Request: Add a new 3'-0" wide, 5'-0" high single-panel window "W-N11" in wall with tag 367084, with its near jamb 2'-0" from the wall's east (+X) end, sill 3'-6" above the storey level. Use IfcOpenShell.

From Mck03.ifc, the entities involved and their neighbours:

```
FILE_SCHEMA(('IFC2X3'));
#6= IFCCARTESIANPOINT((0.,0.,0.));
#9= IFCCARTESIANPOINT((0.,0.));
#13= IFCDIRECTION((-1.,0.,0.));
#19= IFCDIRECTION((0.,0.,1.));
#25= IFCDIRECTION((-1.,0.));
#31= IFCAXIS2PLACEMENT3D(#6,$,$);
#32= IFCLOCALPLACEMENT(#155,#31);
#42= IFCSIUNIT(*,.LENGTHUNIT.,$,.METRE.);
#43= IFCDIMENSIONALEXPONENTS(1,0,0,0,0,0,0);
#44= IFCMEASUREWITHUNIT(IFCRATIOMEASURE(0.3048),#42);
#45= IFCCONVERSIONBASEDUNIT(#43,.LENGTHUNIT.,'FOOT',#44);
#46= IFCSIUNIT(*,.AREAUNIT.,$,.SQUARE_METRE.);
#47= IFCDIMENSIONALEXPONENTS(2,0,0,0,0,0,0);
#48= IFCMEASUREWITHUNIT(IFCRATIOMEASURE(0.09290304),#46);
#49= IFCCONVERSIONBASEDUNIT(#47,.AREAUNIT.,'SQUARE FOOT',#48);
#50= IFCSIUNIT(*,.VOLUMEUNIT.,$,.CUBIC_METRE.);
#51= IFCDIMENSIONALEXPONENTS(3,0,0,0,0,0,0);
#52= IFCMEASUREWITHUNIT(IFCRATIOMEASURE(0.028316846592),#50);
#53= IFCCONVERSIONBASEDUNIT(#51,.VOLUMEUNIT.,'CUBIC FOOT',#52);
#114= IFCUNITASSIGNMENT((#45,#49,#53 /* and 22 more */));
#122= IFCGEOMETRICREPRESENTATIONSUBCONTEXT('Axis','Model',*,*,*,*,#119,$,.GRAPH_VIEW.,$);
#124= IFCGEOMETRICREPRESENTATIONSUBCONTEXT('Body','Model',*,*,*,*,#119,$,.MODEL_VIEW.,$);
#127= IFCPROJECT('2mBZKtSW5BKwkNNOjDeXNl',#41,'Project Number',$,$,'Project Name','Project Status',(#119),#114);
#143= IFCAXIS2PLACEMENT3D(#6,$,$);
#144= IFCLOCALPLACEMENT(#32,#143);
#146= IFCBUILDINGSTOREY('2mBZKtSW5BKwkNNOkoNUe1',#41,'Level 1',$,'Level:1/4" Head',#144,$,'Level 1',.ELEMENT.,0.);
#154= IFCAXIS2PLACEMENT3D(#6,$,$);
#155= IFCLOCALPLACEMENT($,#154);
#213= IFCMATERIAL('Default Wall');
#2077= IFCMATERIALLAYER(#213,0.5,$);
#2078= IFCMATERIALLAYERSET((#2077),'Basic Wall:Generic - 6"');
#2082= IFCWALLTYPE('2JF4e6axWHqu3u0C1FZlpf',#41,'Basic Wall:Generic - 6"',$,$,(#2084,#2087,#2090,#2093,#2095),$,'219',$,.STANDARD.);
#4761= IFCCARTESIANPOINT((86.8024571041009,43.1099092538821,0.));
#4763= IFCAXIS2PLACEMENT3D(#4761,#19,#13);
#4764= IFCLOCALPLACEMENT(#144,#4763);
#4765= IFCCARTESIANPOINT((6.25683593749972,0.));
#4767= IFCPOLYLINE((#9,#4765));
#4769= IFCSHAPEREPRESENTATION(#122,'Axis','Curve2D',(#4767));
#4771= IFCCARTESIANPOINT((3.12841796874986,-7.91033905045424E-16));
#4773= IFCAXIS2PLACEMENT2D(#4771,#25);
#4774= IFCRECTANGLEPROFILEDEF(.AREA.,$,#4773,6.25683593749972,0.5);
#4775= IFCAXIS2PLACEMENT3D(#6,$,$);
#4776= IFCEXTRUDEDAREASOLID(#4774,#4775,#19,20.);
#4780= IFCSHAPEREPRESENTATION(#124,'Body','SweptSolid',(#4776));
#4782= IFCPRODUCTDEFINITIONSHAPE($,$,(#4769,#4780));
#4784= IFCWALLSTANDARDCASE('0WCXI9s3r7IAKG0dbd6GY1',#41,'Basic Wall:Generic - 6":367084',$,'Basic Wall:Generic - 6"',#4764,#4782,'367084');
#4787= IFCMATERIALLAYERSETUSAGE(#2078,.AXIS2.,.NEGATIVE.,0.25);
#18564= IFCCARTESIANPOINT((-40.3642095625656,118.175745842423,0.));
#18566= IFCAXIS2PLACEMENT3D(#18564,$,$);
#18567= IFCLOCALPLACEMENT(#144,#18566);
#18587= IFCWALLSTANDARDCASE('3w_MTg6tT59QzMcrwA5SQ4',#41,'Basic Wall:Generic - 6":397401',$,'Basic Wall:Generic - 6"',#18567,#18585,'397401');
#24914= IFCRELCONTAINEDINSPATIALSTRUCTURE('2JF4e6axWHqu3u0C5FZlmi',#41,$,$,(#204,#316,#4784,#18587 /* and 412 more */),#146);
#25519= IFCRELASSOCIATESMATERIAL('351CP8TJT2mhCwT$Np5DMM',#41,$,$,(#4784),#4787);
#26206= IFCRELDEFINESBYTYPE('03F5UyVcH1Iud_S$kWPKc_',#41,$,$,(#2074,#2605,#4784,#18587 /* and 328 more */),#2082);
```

```python
import numpy as np
import ifcopenshell
import ifcopenshell.api.feature
import ifcopenshell.api.geometry
import ifcopenshell.api.root
import ifcopenshell.api.spatial
import ifcopenshell.api.type
import ifcopenshell.geom
import ifcopenshell.util.element
import ifcopenshell.util.placement
import ifcopenshell.util.representation
import ifcopenshell.util.shape
import ifcopenshell.util.unit

model = ifcopenshell.open("Mck03.ifc")
unit_scale = ifcopenshell.util.unit.calculate_unit_scale(model)
settings = ifcopenshell.geom.settings()


def volume(element):
    """Net volume in cubic metres, openings subtracted."""
    shape = ifcopenshell.geom.create_shape(settings, element)
    return ifcopenshell.util.shape.get_volume(shape.geometry)


wall = model.by_guid("0WCXI9s3r7IAKG0dbd6GY1")
storey = ifcopenshell.util.element.get_container(wall, ifc_class="IfcBuildingStorey")
context = ifcopenshell.util.representation.get_context(model, "Model", "Body", "MODEL_VIEW")
before = volume(wall)

width, height, from_end, sill = 0.9144, 1.524, 0.6096, 1.0668  # metres

# The wall runs along its own X axis, and the end named is its -X end.
wall_shape = ifcopenshell.geom.create_shape(settings, wall)
x, y, z = ifcopenshell.util.shape.get_vertices(wall_shape.geometry).T
start = x.min() + from_end
face, thickness = float(y.min()), float(y.max() - y.min())
wall_matrix = ifcopenshell.util.placement.get_local_placement(wall.ObjectPlacement)
level = ifcopenshell.util.placement.get_local_placement(storey.ObjectPlacement)[2, 3]


def in_wall(x, y):
    """Placement at x, y metres in the wall's axes, at sill height."""
    matrix = wall_matrix.copy()
    matrix[:, 3] = wall_matrix @ np.array([x / unit_scale, y / unit_scale, 0.0, 1.0])
    matrix[2, 3] = level + sill / unit_scale
    return matrix


# Opening: a box that overshoots both wall faces by 50 mm.
opening = ifcopenshell.api.root.create_entity(model, ifc_class="IfcOpeningElement")
box = ifcopenshell.api.geometry.add_wall_representation(
    model, context=context, length=width, height=height, thickness=thickness + 0.1
)
ifcopenshell.api.geometry.assign_representation(model, product=opening, representation=box)
ifcopenshell.api.geometry.edit_object_placement(model, product=opening, matrix=in_wall(start, face - 0.05), is_si=False)
ifcopenshell.api.feature.add_feature(model, feature=opening, element=wall)

window = ifcopenshell.api.root.create_entity(model, ifc_class="IfcWindow", name="W-N11")
window.OverallWidth, window.OverallHeight = width / unit_scale, height / unit_scale
body = ifcopenshell.api.geometry.add_window_representation(
    model,
    context=context,
    overall_width=window.OverallWidth,
    overall_height=window.OverallHeight,
    partition_type="SINGLE_PANEL",
)
ifcopenshell.api.geometry.assign_representation(model, product=window, representation=body)
ifcopenshell.api.spatial.assign_container(model, products=[window], relating_structure=storey)
fills = ifcopenshell.api.feature.add_filling(model, opening=opening, element=window)
fills.OwnerHistory = window.OwnerHistory  # required in IFC2X3

# IFC2X3 keeps the operation on the window style.
style = ifcopenshell.api.root.create_entity(model, ifc_class="IfcWindowStyle", name="W-N11")
style.OperationType, style.ConstructionType = "SINGLE_PANEL", "NOTDEFINED"
style.ParameterTakesPrecedence = style.Sizeable = False
ifcopenshell.api.type.assign_type(model, related_objects=[window], relating_type=style)

# Centre the window in the wall's thickness.
ifcopenshell.api.geometry.edit_object_placement(model, product=window, matrix=in_wall(start, face), is_si=False)
window_shape = ifcopenshell.geom.create_shape(settings, window)
depth = ifcopenshell.util.shape.get_vertices(window_shape.geometry)[:, 1]
offset = face + thickness / 2 - (depth.min() + depth.max()) / 2
ifcopenshell.api.geometry.edit_object_placement(model, product=window, matrix=in_wall(start, offset), is_si=False)

after = volume(wall)

print(f"wall volume {before:.3f} -> {after:.3f} m3")

model.write("Mck03-out.ifc")
```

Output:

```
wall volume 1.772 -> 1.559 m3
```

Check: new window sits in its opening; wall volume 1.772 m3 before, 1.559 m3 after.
